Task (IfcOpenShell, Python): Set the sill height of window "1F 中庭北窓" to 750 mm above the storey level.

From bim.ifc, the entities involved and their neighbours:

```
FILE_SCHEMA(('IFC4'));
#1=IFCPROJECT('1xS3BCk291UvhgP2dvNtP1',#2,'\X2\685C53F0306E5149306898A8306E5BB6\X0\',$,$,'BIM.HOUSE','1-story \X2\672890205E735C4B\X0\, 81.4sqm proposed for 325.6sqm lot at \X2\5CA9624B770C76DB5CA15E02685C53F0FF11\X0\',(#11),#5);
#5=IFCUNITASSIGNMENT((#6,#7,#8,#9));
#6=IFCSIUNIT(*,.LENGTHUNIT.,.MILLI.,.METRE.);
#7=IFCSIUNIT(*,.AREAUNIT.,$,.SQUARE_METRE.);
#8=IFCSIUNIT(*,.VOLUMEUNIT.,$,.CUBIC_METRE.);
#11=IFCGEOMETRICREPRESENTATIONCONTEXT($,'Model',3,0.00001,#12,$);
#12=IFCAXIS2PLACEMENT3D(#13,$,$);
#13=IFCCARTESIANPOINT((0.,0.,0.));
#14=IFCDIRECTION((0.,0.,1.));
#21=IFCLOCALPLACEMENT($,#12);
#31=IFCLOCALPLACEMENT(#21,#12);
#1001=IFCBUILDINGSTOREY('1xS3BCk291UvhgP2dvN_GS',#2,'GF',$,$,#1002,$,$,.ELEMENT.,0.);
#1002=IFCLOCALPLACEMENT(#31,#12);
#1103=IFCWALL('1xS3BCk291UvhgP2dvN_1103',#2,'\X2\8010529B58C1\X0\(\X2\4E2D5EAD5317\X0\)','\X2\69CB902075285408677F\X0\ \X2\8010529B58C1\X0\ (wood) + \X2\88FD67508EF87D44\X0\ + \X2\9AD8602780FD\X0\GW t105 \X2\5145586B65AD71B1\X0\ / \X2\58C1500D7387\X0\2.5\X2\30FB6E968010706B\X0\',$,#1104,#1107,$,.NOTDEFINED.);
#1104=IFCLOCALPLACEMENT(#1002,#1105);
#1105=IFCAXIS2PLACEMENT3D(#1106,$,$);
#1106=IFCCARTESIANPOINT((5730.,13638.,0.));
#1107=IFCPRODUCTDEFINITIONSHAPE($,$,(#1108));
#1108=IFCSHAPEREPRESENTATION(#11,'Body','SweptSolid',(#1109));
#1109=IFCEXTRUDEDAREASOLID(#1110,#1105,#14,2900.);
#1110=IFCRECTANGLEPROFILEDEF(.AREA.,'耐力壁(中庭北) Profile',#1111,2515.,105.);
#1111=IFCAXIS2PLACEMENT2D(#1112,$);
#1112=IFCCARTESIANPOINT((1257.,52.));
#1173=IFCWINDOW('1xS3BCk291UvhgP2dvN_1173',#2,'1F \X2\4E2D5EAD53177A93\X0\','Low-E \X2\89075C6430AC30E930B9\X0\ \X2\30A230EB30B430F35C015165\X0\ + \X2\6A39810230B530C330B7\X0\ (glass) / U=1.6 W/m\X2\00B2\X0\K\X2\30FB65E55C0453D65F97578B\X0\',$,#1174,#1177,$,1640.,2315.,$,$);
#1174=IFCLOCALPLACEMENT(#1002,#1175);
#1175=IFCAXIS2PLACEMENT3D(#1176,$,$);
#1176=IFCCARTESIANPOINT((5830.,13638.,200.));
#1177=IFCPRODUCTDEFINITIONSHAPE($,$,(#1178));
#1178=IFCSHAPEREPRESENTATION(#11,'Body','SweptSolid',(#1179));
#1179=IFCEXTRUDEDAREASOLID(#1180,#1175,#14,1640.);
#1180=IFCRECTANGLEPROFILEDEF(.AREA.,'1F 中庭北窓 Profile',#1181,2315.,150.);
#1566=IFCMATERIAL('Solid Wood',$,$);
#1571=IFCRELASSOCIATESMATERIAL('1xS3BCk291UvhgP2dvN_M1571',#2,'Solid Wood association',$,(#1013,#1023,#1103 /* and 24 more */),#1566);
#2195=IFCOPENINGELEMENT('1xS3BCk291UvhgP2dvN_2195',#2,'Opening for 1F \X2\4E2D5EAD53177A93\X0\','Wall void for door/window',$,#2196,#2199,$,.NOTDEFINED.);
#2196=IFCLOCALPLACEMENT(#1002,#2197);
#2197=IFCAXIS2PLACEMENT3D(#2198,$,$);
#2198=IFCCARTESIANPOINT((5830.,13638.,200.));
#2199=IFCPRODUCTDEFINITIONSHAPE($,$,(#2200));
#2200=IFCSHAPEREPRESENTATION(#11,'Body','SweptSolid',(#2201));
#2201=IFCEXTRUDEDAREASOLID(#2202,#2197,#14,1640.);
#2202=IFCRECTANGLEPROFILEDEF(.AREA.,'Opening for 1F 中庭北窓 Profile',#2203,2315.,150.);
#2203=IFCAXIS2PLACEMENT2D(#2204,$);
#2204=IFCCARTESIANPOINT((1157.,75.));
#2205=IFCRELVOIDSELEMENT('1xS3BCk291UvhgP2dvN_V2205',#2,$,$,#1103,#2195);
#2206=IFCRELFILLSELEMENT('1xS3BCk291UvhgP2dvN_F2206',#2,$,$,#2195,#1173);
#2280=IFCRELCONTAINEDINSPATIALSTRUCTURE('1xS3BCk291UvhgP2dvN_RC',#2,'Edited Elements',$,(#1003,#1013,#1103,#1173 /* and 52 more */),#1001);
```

```python
import numpy as np
import ifcopenshell
import ifcopenshell.api.geometry
import ifcopenshell.geom
import ifcopenshell.util.element
import ifcopenshell.util.placement
import ifcopenshell.util.shape
import ifcopenshell.util.unit

model = ifcopenshell.open("bim.ifc")
unit_scale = ifcopenshell.util.unit.calculate_unit_scale(model)

window = model.by_guid("1xS3BCk291UvhgP2dvN_1173")
opening = window.FillsVoids[0].RelatingOpeningElement
storey = ifcopenshell.util.element.get_container(window, ifc_class="IfcBuildingStorey")
level = ifcopenshell.util.placement.get_local_placement(storey.ObjectPlacement)[2, 3]

# The opening's origin need not be at the sill, so measure its lowest point.
shape = ifcopenshell.geom.create_shape(ifcopenshell.geom.settings(), opening)
bottom = ifcopenshell.util.shape.get_shape_bottom_elevation(shape, shape.geometry) / unit_scale
dz = level + 750.0 - bottom

shift = np.array([0.0, 0.0, dz])
# The window is not placed relative to its opening, so move both.
for product in (opening, window):
    matrix = ifcopenshell.util.placement.get_local_placement(product.ObjectPlacement)
    matrix[:3, 3] += shift
    ifcopenshell.api.geometry.edit_object_placement(model, product=product, matrix=matrix, is_si=False)

print(f"moved by {dz * unit_scale:+.3f} m")

model.write("bim-out.ifc")
```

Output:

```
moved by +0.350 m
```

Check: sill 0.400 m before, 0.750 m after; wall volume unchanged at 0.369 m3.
